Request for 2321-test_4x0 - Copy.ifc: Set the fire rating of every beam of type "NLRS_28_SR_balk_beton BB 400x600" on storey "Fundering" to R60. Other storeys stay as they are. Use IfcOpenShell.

First a look at what the model holds.

```python
import ifcopenshell
import ifcopenshell.util.element

model = ifcopenshell.open("2321-test_4x0 - Copy.ifc")
print(model.schema)
storey = next(s for s in model.by_type("IfcBuildingStorey") if s.Name == "Fundering")
beams = [e for e in ifcopenshell.util.element.get_decomposition(storey) if e.is_a("IfcBeam")]
seen = {}
for e in beams:
    element_type = ifcopenshell.util.element.get_type(e)
    key = (element_type.Name if element_type != e and element_type else None, ifcopenshell.util.element.get_pset(e, "Pset_BeamCommon", "FireRating"))
    seen[key] = seen.get(key, 0) + 1
for (name, value), count in sorted(seen.items(), key=str):
    print(count, "x", name, "|", value)
```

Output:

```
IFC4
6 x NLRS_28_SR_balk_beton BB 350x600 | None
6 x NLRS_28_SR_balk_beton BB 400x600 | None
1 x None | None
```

```python
import ifcopenshell
import ifcopenshell.api.pset
import ifcopenshell.util.element

model = ifcopenshell.open("2321-test_4x0 - Copy.ifc")

storey = next(s for s in model.by_type("IfcBuildingStorey") if s.Name == "Fundering")
beams = [e for e in ifcopenshell.util.element.get_decomposition(storey) if e.is_a("IfcBeam")]

count = 0
for e in beams:
    element_type = ifcopenshell.util.element.get_type(e)
    if element_type in (None, e) or element_type.Name != "NLRS_28_SR_balk_beton BB 400x600":
        continue
    # add_pset returns the element's existing set when there is one.
    pset = ifcopenshell.api.pset.add_pset(model, product=e, name="Pset_BeamCommon")
    ifcopenshell.api.pset.edit_pset(model, pset=pset, properties={"FireRating": "R60"})
    count += 1

print(count, "beams updated")

model.write("2321-test_4x0 - Copy_updated.ifc")
```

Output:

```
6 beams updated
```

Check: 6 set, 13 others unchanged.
